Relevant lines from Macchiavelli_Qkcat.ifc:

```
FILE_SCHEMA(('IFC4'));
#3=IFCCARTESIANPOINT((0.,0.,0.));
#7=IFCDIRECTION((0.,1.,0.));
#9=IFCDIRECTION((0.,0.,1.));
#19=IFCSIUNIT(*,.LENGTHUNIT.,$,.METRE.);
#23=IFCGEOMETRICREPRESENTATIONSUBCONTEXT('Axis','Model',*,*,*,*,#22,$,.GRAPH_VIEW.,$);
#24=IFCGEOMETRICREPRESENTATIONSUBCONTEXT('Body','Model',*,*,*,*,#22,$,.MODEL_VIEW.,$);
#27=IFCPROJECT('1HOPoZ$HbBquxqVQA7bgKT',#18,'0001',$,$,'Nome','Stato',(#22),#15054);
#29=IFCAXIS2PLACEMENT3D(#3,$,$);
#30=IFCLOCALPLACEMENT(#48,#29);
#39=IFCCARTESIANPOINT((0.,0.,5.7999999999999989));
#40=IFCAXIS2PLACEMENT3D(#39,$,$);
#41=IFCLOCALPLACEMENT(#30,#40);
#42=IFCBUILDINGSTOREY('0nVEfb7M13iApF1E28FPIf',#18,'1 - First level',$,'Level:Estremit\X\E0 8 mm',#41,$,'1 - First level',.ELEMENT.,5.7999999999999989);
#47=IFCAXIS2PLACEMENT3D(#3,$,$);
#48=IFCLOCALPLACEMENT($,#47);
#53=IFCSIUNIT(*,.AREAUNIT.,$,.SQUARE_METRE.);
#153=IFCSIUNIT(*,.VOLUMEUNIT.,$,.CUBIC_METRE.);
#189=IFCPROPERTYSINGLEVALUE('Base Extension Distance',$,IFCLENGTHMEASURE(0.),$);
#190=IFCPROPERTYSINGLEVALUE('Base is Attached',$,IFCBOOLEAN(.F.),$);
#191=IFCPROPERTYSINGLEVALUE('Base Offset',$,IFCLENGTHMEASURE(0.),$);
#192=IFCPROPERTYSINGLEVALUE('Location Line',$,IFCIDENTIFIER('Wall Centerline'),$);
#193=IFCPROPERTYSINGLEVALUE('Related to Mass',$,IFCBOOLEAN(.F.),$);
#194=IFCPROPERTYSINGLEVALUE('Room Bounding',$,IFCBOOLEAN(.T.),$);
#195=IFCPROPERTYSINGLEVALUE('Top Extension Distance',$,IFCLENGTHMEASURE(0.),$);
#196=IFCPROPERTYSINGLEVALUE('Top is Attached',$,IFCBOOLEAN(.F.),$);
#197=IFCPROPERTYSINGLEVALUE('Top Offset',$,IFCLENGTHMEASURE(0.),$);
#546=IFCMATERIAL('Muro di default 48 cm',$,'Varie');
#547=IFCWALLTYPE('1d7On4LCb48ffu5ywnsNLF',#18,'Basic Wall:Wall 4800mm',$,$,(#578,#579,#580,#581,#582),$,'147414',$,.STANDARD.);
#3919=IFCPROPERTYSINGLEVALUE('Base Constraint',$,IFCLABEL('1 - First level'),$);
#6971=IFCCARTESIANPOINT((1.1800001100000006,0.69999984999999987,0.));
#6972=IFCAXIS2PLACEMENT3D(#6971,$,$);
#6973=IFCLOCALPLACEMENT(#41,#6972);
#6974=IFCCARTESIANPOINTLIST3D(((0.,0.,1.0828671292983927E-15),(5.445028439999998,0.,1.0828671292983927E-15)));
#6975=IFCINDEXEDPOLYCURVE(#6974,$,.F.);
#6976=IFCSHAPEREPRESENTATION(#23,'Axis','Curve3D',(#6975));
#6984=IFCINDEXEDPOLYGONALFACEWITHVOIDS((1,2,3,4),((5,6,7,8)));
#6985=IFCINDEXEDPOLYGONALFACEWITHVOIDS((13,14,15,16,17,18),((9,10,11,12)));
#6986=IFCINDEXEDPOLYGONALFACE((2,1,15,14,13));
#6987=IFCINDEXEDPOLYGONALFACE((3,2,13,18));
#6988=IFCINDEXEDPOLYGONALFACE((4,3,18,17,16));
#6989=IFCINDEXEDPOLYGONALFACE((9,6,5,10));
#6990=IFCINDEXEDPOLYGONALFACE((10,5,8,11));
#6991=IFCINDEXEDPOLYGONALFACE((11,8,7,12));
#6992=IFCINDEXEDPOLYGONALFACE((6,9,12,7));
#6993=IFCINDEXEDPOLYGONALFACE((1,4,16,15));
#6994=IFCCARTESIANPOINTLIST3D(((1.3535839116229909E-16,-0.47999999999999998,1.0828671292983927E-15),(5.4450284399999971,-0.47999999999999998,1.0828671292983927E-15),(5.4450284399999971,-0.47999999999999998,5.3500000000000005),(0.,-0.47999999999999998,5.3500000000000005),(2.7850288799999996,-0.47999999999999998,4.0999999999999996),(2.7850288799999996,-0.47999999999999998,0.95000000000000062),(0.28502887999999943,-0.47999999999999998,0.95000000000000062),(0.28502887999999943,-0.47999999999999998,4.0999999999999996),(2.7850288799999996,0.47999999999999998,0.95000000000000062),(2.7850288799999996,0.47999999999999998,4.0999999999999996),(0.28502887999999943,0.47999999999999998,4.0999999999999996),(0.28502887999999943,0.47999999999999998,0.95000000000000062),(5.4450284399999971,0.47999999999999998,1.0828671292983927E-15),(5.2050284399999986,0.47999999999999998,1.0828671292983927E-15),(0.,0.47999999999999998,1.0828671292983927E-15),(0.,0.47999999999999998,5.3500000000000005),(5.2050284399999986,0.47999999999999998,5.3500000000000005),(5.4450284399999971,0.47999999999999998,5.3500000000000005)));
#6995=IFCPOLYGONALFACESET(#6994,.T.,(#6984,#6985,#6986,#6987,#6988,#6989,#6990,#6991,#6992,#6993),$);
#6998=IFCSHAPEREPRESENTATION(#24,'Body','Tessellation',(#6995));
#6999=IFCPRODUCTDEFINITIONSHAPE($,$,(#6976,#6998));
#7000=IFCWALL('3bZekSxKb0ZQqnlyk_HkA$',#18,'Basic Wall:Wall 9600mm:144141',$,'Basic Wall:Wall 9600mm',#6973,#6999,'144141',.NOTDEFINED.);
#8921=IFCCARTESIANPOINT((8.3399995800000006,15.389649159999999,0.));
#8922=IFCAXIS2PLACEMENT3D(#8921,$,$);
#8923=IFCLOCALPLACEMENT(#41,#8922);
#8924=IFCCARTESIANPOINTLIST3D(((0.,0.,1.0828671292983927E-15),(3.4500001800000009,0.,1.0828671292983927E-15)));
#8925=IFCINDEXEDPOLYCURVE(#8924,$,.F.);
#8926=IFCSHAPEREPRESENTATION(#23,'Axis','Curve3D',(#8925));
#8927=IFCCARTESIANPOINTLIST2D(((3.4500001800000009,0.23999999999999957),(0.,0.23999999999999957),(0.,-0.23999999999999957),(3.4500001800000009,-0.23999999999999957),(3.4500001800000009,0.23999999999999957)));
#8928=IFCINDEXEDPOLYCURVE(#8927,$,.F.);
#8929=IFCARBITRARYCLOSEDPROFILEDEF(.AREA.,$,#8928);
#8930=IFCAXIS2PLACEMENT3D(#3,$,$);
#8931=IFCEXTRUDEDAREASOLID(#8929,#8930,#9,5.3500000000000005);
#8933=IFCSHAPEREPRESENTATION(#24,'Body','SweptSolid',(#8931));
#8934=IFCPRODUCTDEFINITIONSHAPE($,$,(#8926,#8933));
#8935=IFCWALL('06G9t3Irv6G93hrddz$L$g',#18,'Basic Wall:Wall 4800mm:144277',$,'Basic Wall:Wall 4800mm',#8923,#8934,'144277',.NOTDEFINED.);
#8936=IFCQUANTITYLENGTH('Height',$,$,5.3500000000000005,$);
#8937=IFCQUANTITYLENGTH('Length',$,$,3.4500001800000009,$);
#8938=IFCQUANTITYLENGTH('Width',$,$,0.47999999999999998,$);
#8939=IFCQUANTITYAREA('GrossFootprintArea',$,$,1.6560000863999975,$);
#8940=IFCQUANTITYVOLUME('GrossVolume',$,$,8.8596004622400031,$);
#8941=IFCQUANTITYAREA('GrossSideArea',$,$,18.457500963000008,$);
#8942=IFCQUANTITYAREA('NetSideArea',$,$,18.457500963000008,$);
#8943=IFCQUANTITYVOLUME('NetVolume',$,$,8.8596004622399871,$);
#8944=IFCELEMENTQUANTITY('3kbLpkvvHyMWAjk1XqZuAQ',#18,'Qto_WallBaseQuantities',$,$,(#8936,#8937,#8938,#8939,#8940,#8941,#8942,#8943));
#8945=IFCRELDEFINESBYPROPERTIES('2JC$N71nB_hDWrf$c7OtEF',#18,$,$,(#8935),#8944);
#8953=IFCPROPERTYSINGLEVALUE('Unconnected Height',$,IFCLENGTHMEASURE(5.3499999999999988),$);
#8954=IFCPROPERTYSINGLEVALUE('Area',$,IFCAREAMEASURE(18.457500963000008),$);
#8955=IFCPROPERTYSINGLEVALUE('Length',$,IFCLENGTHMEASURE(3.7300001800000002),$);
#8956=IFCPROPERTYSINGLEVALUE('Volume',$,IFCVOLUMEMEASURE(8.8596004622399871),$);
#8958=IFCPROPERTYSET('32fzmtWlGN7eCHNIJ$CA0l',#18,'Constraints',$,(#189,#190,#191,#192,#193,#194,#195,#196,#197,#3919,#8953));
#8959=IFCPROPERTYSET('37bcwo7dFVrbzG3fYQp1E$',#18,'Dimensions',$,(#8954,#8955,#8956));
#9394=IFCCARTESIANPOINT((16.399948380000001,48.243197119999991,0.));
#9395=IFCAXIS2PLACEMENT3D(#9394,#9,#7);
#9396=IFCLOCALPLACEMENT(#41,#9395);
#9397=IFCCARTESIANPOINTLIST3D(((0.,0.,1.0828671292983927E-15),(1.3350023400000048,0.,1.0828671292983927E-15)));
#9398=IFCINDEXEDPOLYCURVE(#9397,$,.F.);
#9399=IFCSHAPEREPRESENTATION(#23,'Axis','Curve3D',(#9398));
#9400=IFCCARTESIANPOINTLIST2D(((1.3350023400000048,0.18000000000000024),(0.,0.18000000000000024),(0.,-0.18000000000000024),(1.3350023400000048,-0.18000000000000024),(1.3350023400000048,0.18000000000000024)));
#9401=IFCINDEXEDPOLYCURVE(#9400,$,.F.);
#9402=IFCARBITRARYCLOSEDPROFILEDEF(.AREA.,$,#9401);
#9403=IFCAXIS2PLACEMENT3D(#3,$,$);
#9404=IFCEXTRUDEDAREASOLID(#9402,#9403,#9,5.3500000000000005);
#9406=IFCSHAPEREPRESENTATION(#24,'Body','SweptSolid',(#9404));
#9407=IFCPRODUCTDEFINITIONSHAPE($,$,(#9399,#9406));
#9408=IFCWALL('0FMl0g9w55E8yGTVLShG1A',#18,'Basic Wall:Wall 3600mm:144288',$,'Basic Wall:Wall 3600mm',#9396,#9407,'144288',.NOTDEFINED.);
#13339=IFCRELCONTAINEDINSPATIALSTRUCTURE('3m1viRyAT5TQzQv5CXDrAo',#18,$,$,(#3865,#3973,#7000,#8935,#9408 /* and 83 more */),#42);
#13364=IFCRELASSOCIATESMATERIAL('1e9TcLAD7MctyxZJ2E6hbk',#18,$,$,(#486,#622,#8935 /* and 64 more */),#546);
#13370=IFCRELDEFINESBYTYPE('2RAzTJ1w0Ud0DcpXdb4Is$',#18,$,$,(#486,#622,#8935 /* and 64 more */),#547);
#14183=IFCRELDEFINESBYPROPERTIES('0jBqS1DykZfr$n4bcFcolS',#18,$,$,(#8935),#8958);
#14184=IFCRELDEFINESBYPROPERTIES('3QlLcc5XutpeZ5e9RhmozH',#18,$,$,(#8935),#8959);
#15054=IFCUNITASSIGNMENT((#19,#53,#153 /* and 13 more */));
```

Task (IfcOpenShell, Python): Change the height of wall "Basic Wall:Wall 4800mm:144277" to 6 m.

```python
import ifcopenshell
import ifcopenshell.api.pset
import ifcopenshell.geom
import ifcopenshell.util.element
import ifcopenshell.util.representation
import ifcopenshell.util.shape
import ifcopenshell.util.unit

model = ifcopenshell.open("Macchiavelli_Qkcat.ifc")
unit_scale = ifcopenshell.util.unit.calculate_unit_scale(model)
area_scale = ifcopenshell.util.unit.calculate_unit_scale(model, "AREAUNIT")
volume_scale = ifcopenshell.util.unit.calculate_unit_scale(model, "VOLUMEUNIT")
settings = ifcopenshell.geom.settings()


def volume(element):
    """Net volume in cubic metres, openings subtracted."""
    shape = ifcopenshell.geom.create_shape(settings, element)
    return ifcopenshell.util.shape.get_volume(shape.geometry)


wall = model.by_guid("06G9t3Irv6G93hrddz$L$g")
before = volume(wall)

body = ifcopenshell.util.representation.get_representation(wall, "Model", "Body")
solid = body.Items[0]
old_height = solid.Depth
solid.Depth = 6 / unit_scale
after = volume(wall)
thickness = 0.48  # wall thickness in metres

# Update the stored height, areas and volumes.
qto = model.by_id(ifcopenshell.util.element.get_pset(wall, "Qto_WallBaseQuantities", should_inherit=False)["id"])
ifcopenshell.api.pset.edit_qto(model, qto=qto, properties={
    "Height": solid.Depth,
    "GrossVolume": ifcopenshell.util.element.get_pset(wall, "Qto_WallBaseQuantities", "GrossVolume") * solid.Depth / old_height,
    "GrossSideArea": ifcopenshell.util.element.get_pset(wall, "Qto_WallBaseQuantities", "GrossSideArea") * solid.Depth / old_height,
    "NetSideArea": after / thickness / area_scale,
    "NetVolume": after / volume_scale,
})
pset = model.by_id(ifcopenshell.util.element.get_pset(wall, "Constraints", should_inherit=False)["id"])
ifcopenshell.api.pset.edit_pset(model, pset=pset, properties={
    "Unconnected Height": model.create_entity("IfcLengthMeasure", solid.Depth),
})
pset = model.by_id(ifcopenshell.util.element.get_pset(wall, "Dimensions", should_inherit=False)["id"])
ifcopenshell.api.pset.edit_pset(model, pset=pset, properties={
    "Area": model.create_entity("IfcAreaMeasure", after / thickness / area_scale),
    "Volume": model.create_entity("IfcVolumeMeasure", after / volume_scale),
})

print(f"height {old_height:g} -> {solid.Depth:g}, volume {before:.3f} -> {after:.3f} m3")

model.write("Macchiavelli_Qkcat_rev.ifc")
```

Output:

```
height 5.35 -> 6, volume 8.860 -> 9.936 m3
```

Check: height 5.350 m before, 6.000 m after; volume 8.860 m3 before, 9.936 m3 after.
